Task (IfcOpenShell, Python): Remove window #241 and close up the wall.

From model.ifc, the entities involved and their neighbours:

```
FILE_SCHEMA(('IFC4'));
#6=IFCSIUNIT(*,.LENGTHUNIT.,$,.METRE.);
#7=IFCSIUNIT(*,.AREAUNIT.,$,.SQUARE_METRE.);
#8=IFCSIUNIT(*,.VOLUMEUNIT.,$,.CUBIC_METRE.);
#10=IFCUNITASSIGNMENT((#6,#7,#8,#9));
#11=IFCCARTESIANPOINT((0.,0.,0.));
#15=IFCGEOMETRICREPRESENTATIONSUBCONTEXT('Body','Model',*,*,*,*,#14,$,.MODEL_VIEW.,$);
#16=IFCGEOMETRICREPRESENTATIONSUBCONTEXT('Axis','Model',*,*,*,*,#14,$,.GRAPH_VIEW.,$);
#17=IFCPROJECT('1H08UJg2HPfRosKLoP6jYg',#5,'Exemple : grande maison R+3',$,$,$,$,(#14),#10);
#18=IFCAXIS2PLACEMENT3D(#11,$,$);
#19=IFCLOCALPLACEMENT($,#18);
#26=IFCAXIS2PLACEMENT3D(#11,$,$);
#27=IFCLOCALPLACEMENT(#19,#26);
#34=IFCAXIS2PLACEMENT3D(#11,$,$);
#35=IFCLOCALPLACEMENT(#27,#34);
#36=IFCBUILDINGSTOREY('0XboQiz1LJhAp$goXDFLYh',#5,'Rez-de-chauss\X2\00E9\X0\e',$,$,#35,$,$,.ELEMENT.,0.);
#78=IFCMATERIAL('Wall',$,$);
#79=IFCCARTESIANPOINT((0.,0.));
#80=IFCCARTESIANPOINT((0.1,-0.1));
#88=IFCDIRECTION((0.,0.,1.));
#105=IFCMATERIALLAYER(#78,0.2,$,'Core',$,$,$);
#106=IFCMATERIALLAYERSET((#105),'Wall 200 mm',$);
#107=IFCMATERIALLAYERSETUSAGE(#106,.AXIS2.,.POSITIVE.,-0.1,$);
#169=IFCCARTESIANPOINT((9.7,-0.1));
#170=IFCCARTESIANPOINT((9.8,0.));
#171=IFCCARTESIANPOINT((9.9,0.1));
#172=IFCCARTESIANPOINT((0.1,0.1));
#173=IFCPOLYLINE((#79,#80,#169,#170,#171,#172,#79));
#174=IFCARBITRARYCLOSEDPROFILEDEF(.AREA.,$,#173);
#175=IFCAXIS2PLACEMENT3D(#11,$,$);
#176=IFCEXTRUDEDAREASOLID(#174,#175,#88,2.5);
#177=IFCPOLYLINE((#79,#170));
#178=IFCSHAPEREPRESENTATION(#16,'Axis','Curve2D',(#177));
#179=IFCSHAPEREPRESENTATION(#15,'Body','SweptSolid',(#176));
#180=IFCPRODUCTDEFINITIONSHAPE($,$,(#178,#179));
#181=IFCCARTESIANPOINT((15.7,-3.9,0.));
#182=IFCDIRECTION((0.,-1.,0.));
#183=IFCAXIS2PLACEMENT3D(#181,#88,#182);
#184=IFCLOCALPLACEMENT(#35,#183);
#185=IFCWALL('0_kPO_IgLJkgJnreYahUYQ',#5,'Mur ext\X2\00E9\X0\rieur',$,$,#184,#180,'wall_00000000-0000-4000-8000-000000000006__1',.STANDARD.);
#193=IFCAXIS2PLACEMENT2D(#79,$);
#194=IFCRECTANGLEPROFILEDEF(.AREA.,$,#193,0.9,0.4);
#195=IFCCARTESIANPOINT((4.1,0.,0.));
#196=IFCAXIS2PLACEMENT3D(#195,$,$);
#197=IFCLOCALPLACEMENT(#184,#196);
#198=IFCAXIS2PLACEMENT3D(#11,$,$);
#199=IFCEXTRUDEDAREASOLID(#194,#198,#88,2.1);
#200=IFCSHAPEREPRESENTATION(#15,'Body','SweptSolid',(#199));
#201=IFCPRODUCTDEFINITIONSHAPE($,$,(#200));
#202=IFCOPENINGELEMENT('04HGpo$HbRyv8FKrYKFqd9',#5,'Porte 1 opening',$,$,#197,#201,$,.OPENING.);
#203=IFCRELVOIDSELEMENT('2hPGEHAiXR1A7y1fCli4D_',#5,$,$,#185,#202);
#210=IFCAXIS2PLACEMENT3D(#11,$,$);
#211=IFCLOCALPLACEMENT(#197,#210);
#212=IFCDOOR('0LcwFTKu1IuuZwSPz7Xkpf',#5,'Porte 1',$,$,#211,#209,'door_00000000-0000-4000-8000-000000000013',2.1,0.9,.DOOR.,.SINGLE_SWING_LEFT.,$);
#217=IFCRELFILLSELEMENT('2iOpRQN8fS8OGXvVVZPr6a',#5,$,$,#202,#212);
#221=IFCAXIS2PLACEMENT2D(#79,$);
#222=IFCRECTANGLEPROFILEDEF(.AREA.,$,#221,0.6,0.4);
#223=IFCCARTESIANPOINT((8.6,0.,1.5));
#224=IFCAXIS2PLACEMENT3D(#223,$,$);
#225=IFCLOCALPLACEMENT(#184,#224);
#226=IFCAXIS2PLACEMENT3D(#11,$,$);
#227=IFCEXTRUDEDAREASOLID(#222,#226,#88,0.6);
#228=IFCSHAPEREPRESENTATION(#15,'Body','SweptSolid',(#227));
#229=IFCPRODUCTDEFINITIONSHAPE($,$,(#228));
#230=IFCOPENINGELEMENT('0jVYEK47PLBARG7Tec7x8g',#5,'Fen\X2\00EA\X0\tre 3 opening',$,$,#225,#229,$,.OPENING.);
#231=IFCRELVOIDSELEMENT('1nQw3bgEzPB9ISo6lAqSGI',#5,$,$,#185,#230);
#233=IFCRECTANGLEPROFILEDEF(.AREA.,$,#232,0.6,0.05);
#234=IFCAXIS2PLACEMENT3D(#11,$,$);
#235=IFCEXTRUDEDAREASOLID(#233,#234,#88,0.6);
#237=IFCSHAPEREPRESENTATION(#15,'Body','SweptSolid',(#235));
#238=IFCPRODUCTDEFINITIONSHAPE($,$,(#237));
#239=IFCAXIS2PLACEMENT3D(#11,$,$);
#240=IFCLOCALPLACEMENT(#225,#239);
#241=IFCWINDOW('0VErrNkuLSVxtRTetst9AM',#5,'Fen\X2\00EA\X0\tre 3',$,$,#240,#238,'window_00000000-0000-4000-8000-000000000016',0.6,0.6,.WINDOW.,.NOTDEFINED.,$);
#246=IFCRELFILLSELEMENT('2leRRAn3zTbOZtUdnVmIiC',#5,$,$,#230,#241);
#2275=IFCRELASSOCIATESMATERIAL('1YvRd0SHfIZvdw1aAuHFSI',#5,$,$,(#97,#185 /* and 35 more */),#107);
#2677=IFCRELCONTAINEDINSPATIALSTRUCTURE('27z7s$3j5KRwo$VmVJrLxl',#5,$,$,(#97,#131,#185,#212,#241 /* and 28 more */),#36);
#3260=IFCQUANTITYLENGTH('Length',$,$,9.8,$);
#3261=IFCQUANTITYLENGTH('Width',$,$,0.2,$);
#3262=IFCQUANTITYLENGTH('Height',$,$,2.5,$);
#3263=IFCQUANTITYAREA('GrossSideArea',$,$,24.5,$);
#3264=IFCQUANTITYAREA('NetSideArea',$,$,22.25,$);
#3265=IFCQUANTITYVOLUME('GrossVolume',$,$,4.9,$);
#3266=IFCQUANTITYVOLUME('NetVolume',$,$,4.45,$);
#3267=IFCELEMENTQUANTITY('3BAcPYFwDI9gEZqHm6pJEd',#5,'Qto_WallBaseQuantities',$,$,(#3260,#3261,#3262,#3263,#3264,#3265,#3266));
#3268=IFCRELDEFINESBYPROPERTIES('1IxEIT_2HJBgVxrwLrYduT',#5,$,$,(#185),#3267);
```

```python
import ifcopenshell
import ifcopenshell.api.feature
import ifcopenshell.api.pset
import ifcopenshell.api.root
import ifcopenshell.geom
import ifcopenshell.util.element
import ifcopenshell.util.shape
import ifcopenshell.util.unit

model = ifcopenshell.open("model.ifc")
area_scale = ifcopenshell.util.unit.calculate_unit_scale(model, "AREAUNIT")
volume_scale = ifcopenshell.util.unit.calculate_unit_scale(model, "VOLUMEUNIT")
settings = ifcopenshell.geom.settings()


def volume(element):
    """Net volume in cubic metres, openings subtracted."""
    shape = ifcopenshell.geom.create_shape(settings, element)
    return ifcopenshell.util.shape.get_volume(shape.geometry)


window = model.by_guid("0VErrNkuLSVxtRTetst9AM")
opening = window.FillsVoids[0].RelatingOpeningElement
wall = opening.VoidsElements[0].RelatingBuildingElement
before = volume(wall)

ifcopenshell.api.root.remove_product(model, product=window)
ifcopenshell.api.feature.remove_feature(model, feature=opening)

after = volume(wall)
thickness = 0.2  # wall thickness in metres

# Update the wall's stored quantities.
qto = model.by_id(ifcopenshell.util.element.get_pset(wall, "Qto_WallBaseQuantities", should_inherit=False)["id"])
ifcopenshell.api.pset.edit_qto(model, qto=qto, properties={
    "NetSideArea": after / thickness / area_scale,
    "NetVolume": after / volume_scale,
})

print(f"wall volume {before:.3f} -> {after:.3f} m3")

model.write("model_updated.ifc")
```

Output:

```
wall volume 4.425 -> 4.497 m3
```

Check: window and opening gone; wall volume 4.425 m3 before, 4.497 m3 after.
